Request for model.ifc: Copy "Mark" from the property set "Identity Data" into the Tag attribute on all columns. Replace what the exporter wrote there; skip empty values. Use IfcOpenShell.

First a look at what the model holds.

```python
import ifcopenshell
import ifcopenshell.util.element

model = ifcopenshell.open("model.ifc")
print(model.schema)
columns = model.by_type("IfcColumn")
print(len(columns), "columns")
for e in columns[:8]:
    source = ifcopenshell.util.element.get_pset(e, "Identity Data", "Mark")
    target = e.Tag
    print(e.id(), repr(source), repr(target), sep=" | ")
```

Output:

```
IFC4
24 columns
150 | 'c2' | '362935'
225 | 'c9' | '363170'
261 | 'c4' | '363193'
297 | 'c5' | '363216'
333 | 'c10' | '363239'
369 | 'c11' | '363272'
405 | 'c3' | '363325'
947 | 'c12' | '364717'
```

```python
import ifcopenshell
import ifcopenshell.util.element

model = ifcopenshell.open("model.ifc")

count = 0
for e in model.by_type("IfcColumn"):
    value = ifcopenshell.util.element.get_pset(e, "Identity Data", "Mark")
    current = e.Tag
    if not value or not value.strip() or current == value:
        continue
    e.Tag = value
    count += 1

print(count, "columns updated")

model.write("model-out.ifc")
```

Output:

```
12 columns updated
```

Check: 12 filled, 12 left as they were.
